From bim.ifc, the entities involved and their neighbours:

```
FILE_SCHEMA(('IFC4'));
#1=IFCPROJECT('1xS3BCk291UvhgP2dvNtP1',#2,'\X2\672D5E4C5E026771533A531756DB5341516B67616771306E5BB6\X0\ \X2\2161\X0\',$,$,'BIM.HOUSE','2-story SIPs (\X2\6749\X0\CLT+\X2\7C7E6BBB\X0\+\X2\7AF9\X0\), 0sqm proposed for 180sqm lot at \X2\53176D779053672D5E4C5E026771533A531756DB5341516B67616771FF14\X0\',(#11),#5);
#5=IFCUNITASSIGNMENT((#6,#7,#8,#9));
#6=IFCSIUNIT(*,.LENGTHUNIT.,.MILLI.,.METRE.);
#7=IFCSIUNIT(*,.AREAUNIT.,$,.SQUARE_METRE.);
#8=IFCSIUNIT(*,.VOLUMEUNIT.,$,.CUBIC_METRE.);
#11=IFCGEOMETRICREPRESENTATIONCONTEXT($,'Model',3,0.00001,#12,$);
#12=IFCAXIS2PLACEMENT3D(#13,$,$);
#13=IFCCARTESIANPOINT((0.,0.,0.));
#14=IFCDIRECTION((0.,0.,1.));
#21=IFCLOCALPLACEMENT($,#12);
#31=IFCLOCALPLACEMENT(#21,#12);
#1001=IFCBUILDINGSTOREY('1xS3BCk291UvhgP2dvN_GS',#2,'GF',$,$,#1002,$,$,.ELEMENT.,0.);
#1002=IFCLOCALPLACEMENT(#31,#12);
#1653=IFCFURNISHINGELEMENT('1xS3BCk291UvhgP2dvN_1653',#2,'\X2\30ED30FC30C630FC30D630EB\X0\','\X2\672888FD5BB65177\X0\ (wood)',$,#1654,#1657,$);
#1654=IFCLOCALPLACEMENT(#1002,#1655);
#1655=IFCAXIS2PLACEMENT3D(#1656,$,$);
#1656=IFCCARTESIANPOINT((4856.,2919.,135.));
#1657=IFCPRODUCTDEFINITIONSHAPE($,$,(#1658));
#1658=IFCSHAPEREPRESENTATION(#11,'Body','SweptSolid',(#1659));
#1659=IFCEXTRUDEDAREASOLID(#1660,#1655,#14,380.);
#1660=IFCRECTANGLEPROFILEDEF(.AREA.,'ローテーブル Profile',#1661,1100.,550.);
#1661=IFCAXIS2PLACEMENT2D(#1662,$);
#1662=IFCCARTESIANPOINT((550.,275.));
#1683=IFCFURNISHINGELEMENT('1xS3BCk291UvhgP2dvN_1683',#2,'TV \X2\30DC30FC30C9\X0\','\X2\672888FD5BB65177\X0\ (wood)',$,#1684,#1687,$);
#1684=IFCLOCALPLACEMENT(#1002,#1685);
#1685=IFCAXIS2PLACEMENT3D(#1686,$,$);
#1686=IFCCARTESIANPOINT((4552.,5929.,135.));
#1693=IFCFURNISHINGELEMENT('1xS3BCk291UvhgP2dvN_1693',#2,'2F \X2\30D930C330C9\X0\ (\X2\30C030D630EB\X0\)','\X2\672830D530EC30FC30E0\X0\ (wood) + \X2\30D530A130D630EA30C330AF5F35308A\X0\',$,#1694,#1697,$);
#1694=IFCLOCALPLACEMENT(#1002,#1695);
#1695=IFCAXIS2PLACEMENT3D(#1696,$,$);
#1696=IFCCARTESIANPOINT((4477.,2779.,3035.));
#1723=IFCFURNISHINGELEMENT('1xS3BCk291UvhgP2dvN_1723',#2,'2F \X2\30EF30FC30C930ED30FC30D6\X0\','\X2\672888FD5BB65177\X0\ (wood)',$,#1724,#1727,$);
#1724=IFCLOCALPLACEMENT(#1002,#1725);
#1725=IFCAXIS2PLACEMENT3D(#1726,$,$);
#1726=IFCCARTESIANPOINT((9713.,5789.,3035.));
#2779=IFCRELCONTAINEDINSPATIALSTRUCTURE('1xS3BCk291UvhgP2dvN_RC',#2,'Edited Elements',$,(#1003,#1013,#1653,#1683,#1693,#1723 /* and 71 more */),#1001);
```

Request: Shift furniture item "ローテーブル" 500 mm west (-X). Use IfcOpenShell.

```python
import ifcopenshell
import ifcopenshell.api.geometry
import ifcopenshell.util.placement
import ifcopenshell.util.unit

model = ifcopenshell.open("bim.ifc")
unit_scale = ifcopenshell.util.unit.calculate_unit_scale(model)

item = model.by_guid("1xS3BCk291UvhgP2dvN_1653")
matrix = ifcopenshell.util.placement.get_local_placement(item.ObjectPlacement)
matrix[0, 3] -= 0.5 / unit_scale
ifcopenshell.api.geometry.edit_object_placement(model, product=item, matrix=matrix, is_si=False)

print(ifcopenshell.util.placement.get_local_placement(item.ObjectPlacement).round(3) + 0.0)

model.write("bim_v2.ifc")
```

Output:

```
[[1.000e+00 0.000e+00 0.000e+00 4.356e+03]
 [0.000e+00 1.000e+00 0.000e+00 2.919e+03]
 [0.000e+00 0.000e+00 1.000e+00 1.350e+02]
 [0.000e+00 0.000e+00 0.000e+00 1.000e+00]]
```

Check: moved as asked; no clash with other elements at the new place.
